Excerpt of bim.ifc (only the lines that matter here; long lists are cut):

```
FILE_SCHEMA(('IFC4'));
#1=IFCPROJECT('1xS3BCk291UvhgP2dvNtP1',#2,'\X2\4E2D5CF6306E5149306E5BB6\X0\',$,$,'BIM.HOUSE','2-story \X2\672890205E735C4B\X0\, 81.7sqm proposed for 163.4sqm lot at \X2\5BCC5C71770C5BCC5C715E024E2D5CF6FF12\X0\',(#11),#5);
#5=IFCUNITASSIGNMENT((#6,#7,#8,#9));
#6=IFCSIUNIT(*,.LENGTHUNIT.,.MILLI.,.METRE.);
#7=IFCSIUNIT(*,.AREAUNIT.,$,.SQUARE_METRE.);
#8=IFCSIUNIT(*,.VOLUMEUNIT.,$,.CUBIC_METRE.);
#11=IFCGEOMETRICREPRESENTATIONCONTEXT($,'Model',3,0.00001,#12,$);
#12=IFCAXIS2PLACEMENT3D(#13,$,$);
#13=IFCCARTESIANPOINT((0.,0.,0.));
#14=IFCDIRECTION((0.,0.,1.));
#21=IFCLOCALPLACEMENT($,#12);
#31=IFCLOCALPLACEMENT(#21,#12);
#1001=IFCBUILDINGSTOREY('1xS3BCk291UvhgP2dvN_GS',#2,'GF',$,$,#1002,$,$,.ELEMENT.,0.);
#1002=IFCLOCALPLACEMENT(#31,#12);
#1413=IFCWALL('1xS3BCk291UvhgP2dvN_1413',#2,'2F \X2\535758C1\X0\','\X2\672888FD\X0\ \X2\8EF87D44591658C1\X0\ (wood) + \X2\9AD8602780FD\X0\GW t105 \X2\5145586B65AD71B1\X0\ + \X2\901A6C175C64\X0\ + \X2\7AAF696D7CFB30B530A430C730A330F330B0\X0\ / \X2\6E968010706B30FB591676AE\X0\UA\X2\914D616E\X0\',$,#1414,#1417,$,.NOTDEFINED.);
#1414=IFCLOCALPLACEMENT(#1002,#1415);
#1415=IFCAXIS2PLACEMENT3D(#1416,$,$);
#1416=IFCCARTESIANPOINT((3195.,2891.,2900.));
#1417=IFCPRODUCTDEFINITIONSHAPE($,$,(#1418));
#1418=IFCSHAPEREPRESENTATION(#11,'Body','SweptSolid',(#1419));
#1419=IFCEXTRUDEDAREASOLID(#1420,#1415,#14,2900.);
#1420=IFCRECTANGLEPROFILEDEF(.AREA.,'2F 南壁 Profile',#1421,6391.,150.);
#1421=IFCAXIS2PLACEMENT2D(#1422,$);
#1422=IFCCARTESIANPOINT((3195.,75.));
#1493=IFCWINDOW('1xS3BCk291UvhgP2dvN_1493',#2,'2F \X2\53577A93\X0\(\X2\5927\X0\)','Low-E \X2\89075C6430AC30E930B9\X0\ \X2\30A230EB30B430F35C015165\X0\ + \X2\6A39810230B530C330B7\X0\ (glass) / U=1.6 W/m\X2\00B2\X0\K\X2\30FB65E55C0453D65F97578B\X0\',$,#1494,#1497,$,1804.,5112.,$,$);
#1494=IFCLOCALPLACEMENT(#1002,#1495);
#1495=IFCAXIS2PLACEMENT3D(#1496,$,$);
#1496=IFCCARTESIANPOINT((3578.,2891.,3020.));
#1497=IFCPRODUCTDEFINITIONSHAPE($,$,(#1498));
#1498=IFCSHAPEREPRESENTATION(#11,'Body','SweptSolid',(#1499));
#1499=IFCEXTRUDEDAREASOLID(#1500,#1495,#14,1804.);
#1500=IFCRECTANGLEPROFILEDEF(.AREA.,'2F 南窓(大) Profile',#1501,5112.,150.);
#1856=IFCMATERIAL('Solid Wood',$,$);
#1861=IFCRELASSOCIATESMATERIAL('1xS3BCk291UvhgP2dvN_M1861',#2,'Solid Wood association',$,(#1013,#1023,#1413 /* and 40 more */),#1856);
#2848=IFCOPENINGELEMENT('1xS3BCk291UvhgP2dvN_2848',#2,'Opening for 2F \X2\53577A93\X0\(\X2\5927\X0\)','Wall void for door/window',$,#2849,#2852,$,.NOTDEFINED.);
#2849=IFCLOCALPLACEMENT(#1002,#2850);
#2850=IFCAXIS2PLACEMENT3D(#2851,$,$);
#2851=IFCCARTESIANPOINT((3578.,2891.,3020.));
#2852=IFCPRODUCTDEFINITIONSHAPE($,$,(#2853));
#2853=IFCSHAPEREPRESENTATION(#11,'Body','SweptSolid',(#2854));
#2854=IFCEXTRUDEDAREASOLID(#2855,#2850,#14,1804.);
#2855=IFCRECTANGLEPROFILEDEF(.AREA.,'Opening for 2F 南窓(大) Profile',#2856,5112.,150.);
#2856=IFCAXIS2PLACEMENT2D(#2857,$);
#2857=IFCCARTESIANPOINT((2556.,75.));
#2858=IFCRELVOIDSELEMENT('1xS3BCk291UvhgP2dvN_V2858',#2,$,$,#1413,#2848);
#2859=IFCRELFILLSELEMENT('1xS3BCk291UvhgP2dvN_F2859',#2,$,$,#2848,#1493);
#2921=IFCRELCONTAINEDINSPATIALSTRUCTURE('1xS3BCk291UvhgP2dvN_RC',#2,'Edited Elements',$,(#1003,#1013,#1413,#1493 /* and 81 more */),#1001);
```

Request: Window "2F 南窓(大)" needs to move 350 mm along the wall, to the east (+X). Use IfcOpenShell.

```python
import ifcopenshell
import ifcopenshell.api.geometry
import ifcopenshell.util.placement

model = ifcopenshell.open("bim.ifc")

window = model.by_guid("1xS3BCk291UvhgP2dvN_1493")
opening = window.FillsVoids[0].RelatingOpeningElement
wall = opening.VoidsElements[0].RelatingBuildingElement

wall_matrix = ifcopenshell.util.placement.get_local_placement(wall.ObjectPlacement)
shift = wall_matrix[:3, 0] * 350.0
before = ifcopenshell.util.placement.get_local_placement(window.ObjectPlacement)[:3, 3].copy()

# The window is not placed relative to its opening, so move both.
for product in (opening, window):
    matrix = ifcopenshell.util.placement.get_local_placement(product.ObjectPlacement)
    matrix[:3, 3] += shift
    ifcopenshell.api.geometry.edit_object_placement(model, product=product, matrix=matrix, is_si=False)

after = ifcopenshell.util.placement.get_local_placement(window.ObjectPlacement)[:3, 3]
print("window moved by", (after - before).round(3) + 0.0)

model.write("bim_updated.ifc")
```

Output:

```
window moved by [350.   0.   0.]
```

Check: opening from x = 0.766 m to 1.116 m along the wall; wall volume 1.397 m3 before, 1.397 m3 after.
